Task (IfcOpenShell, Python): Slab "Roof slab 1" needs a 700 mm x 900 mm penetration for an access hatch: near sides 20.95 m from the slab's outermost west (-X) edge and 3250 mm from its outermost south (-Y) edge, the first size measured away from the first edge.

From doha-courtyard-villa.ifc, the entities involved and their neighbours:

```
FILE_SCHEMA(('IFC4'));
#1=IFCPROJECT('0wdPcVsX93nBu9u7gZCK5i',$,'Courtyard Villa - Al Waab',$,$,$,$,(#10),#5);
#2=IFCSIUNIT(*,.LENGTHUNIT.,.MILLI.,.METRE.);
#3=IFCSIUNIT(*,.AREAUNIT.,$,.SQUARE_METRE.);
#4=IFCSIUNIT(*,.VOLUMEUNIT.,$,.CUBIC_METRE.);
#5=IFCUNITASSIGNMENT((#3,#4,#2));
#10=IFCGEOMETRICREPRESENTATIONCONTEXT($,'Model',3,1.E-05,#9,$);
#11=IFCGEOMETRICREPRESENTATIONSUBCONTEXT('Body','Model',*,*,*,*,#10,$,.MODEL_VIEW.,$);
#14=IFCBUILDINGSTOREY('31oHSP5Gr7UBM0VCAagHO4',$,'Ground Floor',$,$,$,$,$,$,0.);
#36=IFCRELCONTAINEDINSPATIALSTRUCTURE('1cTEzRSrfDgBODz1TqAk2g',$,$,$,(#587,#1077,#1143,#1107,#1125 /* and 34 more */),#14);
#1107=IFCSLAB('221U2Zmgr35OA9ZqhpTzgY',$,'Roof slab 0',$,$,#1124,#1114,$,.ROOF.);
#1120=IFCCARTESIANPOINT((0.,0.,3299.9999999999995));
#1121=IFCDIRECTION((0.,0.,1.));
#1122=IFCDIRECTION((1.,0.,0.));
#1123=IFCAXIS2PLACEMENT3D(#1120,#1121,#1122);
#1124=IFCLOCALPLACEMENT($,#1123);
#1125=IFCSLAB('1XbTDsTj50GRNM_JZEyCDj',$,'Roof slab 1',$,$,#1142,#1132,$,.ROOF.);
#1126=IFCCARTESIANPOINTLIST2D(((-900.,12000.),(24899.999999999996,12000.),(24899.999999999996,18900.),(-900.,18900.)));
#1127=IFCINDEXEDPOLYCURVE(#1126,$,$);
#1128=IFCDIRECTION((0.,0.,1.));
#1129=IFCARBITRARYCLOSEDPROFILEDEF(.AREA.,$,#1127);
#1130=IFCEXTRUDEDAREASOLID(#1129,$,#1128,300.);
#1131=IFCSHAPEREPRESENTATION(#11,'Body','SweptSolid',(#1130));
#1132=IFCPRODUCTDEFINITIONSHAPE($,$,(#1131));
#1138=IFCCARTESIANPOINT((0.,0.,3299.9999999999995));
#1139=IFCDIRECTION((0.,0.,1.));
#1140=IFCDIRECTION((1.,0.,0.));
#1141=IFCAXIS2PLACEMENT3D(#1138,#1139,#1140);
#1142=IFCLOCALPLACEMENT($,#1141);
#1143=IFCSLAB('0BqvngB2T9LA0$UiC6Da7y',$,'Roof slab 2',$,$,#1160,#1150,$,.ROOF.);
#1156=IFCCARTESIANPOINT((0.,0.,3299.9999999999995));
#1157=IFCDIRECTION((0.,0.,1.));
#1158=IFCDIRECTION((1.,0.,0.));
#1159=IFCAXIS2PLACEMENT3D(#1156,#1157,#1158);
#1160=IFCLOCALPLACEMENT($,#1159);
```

```python
import numpy as np
import ifcopenshell
import ifcopenshell.api.feature
import ifcopenshell.api.geometry
import ifcopenshell.api.root
import ifcopenshell.geom
import ifcopenshell.util.placement
import ifcopenshell.util.representation
import ifcopenshell.util.shape
import ifcopenshell.util.unit

model = ifcopenshell.open("doha-courtyard-villa.ifc")
unit_scale = ifcopenshell.util.unit.calculate_unit_scale(model)
settings = ifcopenshell.geom.settings()


def volume(element):
    """Net volume in cubic metres, openings subtracted."""
    shape = ifcopenshell.geom.create_shape(settings, element)
    return ifcopenshell.util.shape.get_volume(shape.geometry)


slab = model.by_guid("1XbTDsTj50GRNM_JZEyCDj")
before = volume(slab)

# Extent in the slab's own axes, in metres. The edges named are its -X and -Y sides.
slab_shape = ifcopenshell.geom.create_shape(settings, slab)
vertices = ifcopenshell.util.shape.get_vertices(slab_shape.geometry)
x_min, y_min, bottom = vertices.min(axis=0)
top = vertices[:, 2].max()

opening = ifcopenshell.api.root.create_entity(model, ifc_class="IfcOpeningElement", name="Access hatch opening", predefined_type="OPENING")
context = ifcopenshell.util.representation.get_context(model, "Model", "Body", "MODEL_VIEW")
width, depth = 0.7, 0.9
outline = [(0.0, 0.0), (width, 0.0), (width, depth), (0.0, depth), (0.0, 0.0)]
# Overshoot both faces by 50 mm so the cut is clean.
shape = ifcopenshell.api.geometry.add_slab_representation(
    model, context=context, depth=top - bottom + 0.1, polyline=outline
)
ifcopenshell.api.geometry.assign_representation(model, product=opening, representation=shape)

matrix = ifcopenshell.util.placement.get_local_placement(slab.ObjectPlacement)
matrix[:, 3] = matrix @ np.append(np.array([x_min + 20.95, y_min + 3.25, bottom - 0.05]) / unit_scale, 1.0)
ifcopenshell.api.geometry.edit_object_placement(model, product=opening, matrix=matrix, is_si=False)
ifcopenshell.api.feature.add_feature(model, feature=opening, element=slab)

after = volume(slab)

print(f"slab volume {before:.3f} -> {after:.3f} m3")

model.write("doha-courtyard-villa_v2.ifc")
```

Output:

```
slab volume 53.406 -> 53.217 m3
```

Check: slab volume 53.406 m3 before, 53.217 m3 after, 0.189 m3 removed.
